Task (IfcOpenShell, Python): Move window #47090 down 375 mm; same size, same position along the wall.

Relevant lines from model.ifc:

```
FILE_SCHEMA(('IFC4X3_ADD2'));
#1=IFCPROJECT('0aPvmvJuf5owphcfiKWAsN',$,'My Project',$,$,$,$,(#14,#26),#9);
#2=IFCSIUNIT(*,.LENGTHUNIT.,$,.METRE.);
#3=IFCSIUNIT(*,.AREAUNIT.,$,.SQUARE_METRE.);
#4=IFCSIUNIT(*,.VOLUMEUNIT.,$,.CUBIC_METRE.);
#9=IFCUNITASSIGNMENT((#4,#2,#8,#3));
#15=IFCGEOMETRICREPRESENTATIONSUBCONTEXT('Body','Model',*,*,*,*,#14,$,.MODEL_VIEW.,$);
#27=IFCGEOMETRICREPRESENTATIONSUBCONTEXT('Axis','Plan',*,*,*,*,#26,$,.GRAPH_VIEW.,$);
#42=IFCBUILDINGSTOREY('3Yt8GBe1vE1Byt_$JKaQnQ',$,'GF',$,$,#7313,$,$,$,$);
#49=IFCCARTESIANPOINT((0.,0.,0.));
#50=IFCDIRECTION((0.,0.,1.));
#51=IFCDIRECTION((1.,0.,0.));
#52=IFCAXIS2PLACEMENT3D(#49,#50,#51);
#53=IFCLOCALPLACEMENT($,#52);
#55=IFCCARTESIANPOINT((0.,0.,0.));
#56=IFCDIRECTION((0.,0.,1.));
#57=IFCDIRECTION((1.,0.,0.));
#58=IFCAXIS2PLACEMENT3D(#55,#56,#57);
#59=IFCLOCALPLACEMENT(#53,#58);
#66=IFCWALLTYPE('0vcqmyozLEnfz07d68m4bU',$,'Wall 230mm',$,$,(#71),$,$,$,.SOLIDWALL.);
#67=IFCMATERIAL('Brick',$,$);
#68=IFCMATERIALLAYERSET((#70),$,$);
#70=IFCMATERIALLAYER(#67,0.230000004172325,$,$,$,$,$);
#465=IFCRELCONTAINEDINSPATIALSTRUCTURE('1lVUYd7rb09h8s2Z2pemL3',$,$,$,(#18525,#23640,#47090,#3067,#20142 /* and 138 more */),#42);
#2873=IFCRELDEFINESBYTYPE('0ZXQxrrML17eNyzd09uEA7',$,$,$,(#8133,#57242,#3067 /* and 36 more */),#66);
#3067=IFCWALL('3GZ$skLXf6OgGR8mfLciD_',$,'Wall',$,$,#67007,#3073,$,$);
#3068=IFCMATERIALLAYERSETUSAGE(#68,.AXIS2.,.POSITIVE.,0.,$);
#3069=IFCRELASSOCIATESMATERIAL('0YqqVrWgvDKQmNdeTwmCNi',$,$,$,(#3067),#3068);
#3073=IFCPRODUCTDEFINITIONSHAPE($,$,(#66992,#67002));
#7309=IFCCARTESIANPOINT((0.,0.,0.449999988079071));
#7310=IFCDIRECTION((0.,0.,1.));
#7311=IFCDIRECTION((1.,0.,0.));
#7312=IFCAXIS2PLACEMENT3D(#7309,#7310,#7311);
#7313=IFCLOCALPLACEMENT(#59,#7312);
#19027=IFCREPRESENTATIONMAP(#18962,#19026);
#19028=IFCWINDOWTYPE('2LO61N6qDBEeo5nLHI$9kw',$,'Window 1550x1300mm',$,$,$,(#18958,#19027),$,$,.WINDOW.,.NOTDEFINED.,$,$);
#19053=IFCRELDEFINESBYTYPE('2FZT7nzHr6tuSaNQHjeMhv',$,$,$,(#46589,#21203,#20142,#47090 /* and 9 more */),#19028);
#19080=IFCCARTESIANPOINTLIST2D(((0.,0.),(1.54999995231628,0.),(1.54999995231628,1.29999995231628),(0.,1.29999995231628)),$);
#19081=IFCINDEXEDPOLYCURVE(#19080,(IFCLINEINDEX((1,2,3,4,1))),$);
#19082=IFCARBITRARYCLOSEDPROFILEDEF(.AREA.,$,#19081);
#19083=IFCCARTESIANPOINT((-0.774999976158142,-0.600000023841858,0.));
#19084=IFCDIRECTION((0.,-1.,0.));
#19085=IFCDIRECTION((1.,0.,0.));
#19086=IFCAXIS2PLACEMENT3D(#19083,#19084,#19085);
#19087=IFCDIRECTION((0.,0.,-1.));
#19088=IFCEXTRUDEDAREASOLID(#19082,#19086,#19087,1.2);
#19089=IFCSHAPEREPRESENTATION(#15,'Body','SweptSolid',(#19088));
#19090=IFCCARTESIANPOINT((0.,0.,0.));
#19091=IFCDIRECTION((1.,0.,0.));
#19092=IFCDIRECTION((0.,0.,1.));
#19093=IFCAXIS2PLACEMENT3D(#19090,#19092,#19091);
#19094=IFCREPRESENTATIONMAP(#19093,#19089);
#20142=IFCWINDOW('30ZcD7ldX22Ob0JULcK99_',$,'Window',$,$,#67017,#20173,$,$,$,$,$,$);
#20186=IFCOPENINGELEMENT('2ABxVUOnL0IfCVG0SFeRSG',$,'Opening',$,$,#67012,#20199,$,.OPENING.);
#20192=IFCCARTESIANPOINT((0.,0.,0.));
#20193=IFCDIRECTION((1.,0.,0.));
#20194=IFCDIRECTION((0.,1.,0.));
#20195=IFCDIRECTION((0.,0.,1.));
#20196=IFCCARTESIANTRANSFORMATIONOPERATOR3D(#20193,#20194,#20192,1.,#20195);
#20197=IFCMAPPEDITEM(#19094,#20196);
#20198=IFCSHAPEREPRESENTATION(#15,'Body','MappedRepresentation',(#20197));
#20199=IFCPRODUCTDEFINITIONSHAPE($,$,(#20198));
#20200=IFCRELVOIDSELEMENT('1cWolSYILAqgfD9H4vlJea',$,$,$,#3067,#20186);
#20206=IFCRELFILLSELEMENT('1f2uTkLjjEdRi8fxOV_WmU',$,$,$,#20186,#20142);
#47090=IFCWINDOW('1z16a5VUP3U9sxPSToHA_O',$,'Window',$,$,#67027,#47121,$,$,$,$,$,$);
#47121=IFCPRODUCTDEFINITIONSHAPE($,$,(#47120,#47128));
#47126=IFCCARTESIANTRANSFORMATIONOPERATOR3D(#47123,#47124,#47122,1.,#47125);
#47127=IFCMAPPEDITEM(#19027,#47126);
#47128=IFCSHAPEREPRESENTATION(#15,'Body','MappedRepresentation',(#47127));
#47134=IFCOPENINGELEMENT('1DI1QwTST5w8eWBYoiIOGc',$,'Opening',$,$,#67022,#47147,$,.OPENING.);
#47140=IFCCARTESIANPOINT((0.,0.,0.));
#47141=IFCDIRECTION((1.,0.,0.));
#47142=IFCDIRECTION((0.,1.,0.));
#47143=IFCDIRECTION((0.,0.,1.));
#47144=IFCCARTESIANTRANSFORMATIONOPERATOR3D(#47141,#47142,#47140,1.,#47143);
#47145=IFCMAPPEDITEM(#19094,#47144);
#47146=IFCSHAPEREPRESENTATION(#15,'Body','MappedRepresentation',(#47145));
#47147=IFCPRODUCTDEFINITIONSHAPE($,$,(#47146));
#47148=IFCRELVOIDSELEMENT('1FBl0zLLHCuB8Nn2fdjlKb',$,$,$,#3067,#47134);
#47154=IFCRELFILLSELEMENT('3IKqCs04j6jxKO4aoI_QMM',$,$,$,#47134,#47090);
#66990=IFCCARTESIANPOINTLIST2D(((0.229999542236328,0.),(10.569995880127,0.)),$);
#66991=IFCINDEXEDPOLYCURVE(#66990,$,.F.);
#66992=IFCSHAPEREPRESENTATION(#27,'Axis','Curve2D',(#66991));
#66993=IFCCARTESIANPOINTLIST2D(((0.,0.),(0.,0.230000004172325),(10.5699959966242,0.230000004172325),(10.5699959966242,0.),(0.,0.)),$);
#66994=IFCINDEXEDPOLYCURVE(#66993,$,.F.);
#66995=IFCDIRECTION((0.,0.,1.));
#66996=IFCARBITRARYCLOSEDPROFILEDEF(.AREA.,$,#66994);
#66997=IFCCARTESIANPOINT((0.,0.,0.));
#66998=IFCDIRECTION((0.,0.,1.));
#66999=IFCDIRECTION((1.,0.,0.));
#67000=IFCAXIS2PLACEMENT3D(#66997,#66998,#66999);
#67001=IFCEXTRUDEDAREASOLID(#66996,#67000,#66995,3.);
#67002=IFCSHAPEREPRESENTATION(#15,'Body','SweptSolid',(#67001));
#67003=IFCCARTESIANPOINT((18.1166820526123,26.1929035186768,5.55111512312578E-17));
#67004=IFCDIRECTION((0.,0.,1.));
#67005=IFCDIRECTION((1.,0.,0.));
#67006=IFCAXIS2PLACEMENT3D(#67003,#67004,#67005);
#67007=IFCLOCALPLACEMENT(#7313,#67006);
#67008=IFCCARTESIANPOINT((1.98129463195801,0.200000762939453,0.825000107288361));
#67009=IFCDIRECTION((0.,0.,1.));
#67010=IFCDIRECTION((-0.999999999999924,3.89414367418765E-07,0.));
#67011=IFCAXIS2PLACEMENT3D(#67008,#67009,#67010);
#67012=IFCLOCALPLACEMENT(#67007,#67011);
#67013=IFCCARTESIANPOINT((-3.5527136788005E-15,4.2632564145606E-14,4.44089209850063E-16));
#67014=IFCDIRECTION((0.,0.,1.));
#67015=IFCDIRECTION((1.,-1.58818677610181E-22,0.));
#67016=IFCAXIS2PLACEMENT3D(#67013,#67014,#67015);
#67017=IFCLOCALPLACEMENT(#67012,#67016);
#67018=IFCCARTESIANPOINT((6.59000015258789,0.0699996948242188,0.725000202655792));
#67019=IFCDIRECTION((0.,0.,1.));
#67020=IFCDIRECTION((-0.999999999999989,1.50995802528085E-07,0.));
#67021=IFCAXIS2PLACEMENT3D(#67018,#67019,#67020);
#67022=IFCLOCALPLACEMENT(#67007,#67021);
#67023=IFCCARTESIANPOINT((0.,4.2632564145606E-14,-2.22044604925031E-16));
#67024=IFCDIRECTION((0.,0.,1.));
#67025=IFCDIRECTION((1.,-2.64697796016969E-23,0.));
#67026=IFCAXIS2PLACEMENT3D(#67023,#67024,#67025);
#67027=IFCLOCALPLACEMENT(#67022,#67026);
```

```python
import numpy as np
import ifcopenshell
import ifcopenshell.api.geometry
import ifcopenshell.util.placement
import ifcopenshell.util.unit

model = ifcopenshell.open("model.ifc")
unit_scale = ifcopenshell.util.unit.calculate_unit_scale(model)

window = model.by_id(47090)
opening = window.FillsVoids[0].RelatingOpeningElement
dz = -0.375

shift = np.array([0.0, 0.0, dz])
# The window is placed relative to its opening, so it follows when the opening moves.
matrix = ifcopenshell.util.placement.get_local_placement(opening.ObjectPlacement)
matrix[:3, 3] += shift
ifcopenshell.api.geometry.edit_object_placement(
    model, product=opening, matrix=matrix, is_si=False, should_transform_children=True
)

print(f"moved by {dz * unit_scale:+.3f} m")

model.write("model_rev.ifc")
```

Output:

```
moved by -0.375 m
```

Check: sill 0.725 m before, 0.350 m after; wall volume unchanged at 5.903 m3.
